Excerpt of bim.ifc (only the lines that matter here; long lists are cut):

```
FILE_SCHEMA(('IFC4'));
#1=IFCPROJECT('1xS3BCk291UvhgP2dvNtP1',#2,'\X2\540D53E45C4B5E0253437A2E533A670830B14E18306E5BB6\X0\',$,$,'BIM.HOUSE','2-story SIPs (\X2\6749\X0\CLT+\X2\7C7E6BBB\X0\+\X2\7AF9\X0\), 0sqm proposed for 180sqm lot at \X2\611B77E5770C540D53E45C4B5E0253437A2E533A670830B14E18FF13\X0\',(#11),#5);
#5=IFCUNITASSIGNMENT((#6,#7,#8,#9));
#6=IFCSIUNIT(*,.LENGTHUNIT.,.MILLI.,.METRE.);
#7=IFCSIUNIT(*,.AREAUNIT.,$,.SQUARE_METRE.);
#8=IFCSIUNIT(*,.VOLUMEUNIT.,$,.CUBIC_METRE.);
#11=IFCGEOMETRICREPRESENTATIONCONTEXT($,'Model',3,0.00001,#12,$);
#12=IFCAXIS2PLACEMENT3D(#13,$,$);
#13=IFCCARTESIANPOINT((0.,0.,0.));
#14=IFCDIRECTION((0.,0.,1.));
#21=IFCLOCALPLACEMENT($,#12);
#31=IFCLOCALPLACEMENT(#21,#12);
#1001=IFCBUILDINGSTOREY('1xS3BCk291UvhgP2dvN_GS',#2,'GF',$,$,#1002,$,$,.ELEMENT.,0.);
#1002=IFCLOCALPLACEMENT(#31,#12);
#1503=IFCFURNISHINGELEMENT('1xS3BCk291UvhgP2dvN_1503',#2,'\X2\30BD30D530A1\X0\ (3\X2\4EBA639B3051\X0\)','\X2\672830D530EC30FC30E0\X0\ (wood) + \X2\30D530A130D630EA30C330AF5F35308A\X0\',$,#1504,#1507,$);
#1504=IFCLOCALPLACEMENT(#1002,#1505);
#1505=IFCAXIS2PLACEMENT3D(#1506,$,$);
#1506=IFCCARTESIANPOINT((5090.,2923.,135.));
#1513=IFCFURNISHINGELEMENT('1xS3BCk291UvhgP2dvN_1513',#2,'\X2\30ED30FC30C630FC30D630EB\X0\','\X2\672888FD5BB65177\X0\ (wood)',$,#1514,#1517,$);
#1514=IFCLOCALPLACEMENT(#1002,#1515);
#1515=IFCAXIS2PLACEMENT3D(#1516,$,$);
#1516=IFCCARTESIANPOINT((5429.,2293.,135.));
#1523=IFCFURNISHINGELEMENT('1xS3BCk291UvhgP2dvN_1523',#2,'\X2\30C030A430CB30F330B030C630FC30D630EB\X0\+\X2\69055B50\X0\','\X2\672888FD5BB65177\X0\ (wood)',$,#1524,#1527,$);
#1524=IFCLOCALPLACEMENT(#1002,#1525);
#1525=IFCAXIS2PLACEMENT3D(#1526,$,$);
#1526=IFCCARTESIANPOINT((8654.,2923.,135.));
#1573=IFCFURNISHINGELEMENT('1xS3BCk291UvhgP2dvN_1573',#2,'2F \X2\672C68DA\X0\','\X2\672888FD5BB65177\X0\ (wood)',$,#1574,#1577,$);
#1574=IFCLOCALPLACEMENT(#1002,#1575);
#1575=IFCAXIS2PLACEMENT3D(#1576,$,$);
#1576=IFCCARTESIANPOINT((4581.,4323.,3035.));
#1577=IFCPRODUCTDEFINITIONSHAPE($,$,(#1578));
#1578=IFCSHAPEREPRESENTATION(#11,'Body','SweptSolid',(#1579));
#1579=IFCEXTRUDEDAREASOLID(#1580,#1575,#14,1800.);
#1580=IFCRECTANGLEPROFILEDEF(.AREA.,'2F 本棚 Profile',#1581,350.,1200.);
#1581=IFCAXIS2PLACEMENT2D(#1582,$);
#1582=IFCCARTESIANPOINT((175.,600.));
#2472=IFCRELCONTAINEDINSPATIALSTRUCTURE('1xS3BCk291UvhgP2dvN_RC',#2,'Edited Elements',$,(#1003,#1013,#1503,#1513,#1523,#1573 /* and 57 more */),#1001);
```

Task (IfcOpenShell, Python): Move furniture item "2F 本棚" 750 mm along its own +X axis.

```python
import ifcopenshell
import ifcopenshell.api.geometry
import ifcopenshell.util.placement
import ifcopenshell.util.unit

model = ifcopenshell.open("bim.ifc")
unit_scale = ifcopenshell.util.unit.calculate_unit_scale(model)

item = model.by_guid("1xS3BCk291UvhgP2dvN_1573")
matrix = ifcopenshell.util.placement.get_local_placement(item.ObjectPlacement)
matrix[:3, 3] += matrix[:3, 0] * 0.75 / unit_scale
ifcopenshell.api.geometry.edit_object_placement(model, product=item, matrix=matrix, is_si=False)

print(ifcopenshell.util.placement.get_local_placement(item.ObjectPlacement).round(3) + 0.0)

model.write("bim-out.ifc")
```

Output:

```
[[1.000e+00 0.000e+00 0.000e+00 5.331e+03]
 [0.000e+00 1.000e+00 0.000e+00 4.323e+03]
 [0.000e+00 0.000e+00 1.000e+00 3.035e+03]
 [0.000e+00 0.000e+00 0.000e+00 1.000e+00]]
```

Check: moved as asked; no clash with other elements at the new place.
